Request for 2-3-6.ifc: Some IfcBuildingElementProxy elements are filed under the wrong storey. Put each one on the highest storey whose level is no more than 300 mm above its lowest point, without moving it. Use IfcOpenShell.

First a look at what the model holds.

```python
import ifcopenshell
import ifcopenshell.util.element
import ifcopenshell.util.placement

model = ifcopenshell.open("2-3-6.ifc")
print(model.schema)
for storey in model.by_type("IfcBuildingStorey"):
    level = ifcopenshell.util.placement.get_storey_elevation(storey)
    count = sum(e.is_a("IfcBuildingElementProxy") for e in ifcopenshell.util.element.get_contained(storey))
    print(storey.id(), storey.Name, round(level, 3), count, sep=" | ")
```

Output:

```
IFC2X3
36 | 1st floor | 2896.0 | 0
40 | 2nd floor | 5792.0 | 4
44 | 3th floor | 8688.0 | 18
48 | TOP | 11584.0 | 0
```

```python
import ifcopenshell
import ifcopenshell.api.spatial
import ifcopenshell.geom
import ifcopenshell.util.element
import ifcopenshell.util.placement
import ifcopenshell.util.shape
import ifcopenshell.util.unit

model = ifcopenshell.open("2-3-6.ifc")
unit_scale = ifcopenshell.util.unit.calculate_unit_scale(model)
settings = ifcopenshell.geom.settings()

levels = sorted(
    ((ifcopenshell.util.placement.get_storey_elevation(s) * unit_scale, s) for s in model.by_type("IfcBuildingStorey")),
    key=lambda pair: pair[0],
)

for e in model.by_type("IfcBuildingElementProxy"):
    current = e.ContainedInStructure[0].RelatingStructure if e.ContainedInStructure else None
    if current is None or not current.is_a("IfcBuildingStorey"):
        continue
    shape = ifcopenshell.geom.create_shape(settings, e)
    bottom = ifcopenshell.util.shape.get_shape_bottom_elevation(shape, shape.geometry)
    below = [s for level, s in levels if level <= bottom + 0.3]
    storey = below[-1] if below else levels[0][1]
    if storey != current:
        # assign_container keeps the world position.
        ifcopenshell.api.spatial.assign_container(model, products=[e], relating_structure=storey)
        print(e.id(), current.Name, "->", storey.Name)

model.write("2-3-6_updated.ifc")
```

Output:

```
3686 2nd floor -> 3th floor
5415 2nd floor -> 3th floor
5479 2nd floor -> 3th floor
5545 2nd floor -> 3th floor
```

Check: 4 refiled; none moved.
